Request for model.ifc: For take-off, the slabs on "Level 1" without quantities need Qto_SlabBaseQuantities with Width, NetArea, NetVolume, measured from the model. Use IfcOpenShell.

First a look at what the model holds.

```python
import ifcopenshell
import ifcopenshell.util.element
import ifcopenshell.util.unit

model = ifcopenshell.open("model.ifc")
print(model.schema)
for unit_type in ("LENGTHUNIT", "AREAUNIT", "VOLUMEUNIT"):
    print(unit_type, ifcopenshell.util.unit.calculate_unit_scale(model, unit_type))
storey = next(s for s in model.by_type("IfcBuildingStorey") if s.Name == "Level 1")
slabs = [e for e in ifcopenshell.util.element.get_decomposition(storey) if e.is_a("IfcSlab")]
for e in sorted(slabs, key=lambda e: e.id()):
    print(e.id(), e.is_a(), e.Name, list(ifcopenshell.util.element.get_psets(e, qtos_only=True)), sep=" | ")
```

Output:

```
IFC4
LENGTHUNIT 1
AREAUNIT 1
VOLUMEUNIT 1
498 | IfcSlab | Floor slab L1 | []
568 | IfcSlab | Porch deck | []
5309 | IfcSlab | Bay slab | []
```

```python
import ifcopenshell
import ifcopenshell.api.pset
import ifcopenshell.geom
import ifcopenshell.util.element
import ifcopenshell.util.shape
import ifcopenshell.util.unit

model = ifcopenshell.open("model.ifc")
unit_scale = ifcopenshell.util.unit.calculate_unit_scale(model)
area_scale = ifcopenshell.util.unit.calculate_unit_scale(model, "AREAUNIT")
volume_scale = ifcopenshell.util.unit.calculate_unit_scale(model, "VOLUMEUNIT")
settings = ifcopenshell.geom.settings()

storey = next(s for s in model.by_type("IfcBuildingStorey") if s.Name == "Level 1")
slabs = [e for e in ifcopenshell.util.element.get_decomposition(storey) if e.is_a("IfcSlab")]

for e in sorted(slabs, key=lambda e: e.id()):
    if ifcopenshell.util.element.get_psets(e, qtos_only=True, should_inherit=False):
        continue
    # Geometry comes back in metres, in the element's own axes.
    shape = ifcopenshell.geom.create_shape(settings, e)
    values = {
        "Width": ifcopenshell.util.shape.get_z(shape.geometry) / unit_scale,
        "NetArea": ifcopenshell.util.shape.get_footprint_area(shape.geometry) / area_scale,
        "NetVolume": ifcopenshell.util.shape.get_volume(shape.geometry) / volume_scale,
    }
    qto = ifcopenshell.api.pset.add_qto(model, product=e, name="Qto_SlabBaseQuantities")
    ifcopenshell.api.pset.edit_qto(model, qto=qto, properties=values)
    print(e.id(), {k: round(v, 3) for k, v in values.items()})

model.write("model_rev.ifc")
```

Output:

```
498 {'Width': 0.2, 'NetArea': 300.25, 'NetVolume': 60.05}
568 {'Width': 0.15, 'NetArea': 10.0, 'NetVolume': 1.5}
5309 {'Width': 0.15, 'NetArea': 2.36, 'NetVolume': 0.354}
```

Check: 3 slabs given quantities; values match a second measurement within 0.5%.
